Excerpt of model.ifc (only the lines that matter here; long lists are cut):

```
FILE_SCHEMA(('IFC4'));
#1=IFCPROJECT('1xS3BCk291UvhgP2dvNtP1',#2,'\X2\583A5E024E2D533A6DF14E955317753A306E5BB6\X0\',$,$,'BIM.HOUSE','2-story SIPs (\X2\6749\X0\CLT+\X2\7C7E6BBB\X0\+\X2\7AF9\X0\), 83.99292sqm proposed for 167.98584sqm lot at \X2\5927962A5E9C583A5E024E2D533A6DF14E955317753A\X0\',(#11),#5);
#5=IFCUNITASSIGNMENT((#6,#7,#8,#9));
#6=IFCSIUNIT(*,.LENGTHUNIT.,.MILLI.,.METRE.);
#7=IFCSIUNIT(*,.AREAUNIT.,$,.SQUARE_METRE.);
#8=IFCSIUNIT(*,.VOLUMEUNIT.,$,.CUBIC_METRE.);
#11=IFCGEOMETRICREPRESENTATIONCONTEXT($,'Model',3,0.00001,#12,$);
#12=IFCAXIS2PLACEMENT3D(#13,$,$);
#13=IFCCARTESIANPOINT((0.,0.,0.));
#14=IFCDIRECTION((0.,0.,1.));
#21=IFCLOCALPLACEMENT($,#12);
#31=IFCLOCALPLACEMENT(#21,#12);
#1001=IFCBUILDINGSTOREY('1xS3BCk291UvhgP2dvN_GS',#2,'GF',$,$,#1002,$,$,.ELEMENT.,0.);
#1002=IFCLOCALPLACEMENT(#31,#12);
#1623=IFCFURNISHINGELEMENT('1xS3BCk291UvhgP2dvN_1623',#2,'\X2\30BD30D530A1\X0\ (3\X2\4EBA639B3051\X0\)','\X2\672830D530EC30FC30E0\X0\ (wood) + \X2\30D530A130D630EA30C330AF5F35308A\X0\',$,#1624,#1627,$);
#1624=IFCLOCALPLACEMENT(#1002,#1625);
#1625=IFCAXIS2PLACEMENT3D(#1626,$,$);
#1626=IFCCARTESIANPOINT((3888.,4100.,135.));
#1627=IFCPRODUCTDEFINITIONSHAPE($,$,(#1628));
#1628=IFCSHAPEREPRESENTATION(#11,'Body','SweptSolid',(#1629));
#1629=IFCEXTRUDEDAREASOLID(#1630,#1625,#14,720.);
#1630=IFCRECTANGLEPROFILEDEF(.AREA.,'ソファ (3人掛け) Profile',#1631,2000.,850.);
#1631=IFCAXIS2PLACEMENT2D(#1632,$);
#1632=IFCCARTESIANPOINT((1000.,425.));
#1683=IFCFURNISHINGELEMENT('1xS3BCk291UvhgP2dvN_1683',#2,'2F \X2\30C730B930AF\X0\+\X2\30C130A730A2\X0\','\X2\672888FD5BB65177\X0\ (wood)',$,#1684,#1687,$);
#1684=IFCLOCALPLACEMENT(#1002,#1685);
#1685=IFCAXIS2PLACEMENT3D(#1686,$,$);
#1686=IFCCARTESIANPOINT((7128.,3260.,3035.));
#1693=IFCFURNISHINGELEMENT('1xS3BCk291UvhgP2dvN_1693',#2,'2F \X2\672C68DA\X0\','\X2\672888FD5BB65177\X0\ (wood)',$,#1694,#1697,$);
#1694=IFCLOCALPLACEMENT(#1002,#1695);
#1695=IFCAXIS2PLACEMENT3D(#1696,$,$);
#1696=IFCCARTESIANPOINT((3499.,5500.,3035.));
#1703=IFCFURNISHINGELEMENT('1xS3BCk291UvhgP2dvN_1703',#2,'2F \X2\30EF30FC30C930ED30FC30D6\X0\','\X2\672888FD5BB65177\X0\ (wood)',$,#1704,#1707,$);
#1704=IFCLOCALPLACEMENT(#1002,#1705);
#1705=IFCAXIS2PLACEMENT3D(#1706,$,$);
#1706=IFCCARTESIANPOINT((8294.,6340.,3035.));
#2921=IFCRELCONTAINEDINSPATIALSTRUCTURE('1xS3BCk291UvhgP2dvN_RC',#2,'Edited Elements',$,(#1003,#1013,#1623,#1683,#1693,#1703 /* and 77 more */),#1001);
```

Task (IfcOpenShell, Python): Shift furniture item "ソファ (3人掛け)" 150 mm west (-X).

```python
import ifcopenshell
import ifcopenshell.api.geometry
import ifcopenshell.util.placement

model = ifcopenshell.open("model.ifc")

item = model.by_id(1623)
matrix = ifcopenshell.util.placement.get_local_placement(item.ObjectPlacement)
matrix[0, 3] -= 150.0
ifcopenshell.api.geometry.edit_object_placement(model, product=item, matrix=matrix, is_si=False)

print(ifcopenshell.util.placement.get_local_placement(item.ObjectPlacement).round(3) + 0.0)

model.write("model-out.ifc")
```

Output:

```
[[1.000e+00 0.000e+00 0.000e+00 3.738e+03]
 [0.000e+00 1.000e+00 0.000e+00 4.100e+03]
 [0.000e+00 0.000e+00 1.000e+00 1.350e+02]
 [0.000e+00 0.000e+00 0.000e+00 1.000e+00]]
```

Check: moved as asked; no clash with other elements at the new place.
